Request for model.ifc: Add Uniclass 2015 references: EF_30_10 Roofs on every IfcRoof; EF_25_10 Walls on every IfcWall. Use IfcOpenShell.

First a look at what the model holds.

```python
import ifcopenshell

model = ifcopenshell.open("model.ifc")
print(model.schema)
print("classifications:", [c.Name for c in model.by_type("IfcClassification")])
for ifc_class in ("IfcDoor", "IfcRoof", "IfcStair", "IfcWall", "IfcWindow"):
    print(ifc_class, len(model.by_type(ifc_class)))
```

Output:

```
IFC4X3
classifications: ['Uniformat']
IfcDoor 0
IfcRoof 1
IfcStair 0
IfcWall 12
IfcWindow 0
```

```python
import ifcopenshell
import ifcopenshell.api.classification

model = ifcopenshell.open("model.ifc")

system = ifcopenshell.api.classification.add_classification(model, classification="Uniclass 2015")

codes = {
    "IfcRoof": ("EF_30_10", "Roofs"),
    "IfcWall": ("EF_25_10", "Walls"),
}
for ifc_class, (code, name) in codes.items():
    products = model.by_type(ifc_class)
    ifcopenshell.api.classification.add_reference(
        model, products=products, classification=system, identification=code, name=name
    )
    print(code, len(products))

model.write("model_v2.ifc")
```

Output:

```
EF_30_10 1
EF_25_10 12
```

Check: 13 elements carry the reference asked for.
